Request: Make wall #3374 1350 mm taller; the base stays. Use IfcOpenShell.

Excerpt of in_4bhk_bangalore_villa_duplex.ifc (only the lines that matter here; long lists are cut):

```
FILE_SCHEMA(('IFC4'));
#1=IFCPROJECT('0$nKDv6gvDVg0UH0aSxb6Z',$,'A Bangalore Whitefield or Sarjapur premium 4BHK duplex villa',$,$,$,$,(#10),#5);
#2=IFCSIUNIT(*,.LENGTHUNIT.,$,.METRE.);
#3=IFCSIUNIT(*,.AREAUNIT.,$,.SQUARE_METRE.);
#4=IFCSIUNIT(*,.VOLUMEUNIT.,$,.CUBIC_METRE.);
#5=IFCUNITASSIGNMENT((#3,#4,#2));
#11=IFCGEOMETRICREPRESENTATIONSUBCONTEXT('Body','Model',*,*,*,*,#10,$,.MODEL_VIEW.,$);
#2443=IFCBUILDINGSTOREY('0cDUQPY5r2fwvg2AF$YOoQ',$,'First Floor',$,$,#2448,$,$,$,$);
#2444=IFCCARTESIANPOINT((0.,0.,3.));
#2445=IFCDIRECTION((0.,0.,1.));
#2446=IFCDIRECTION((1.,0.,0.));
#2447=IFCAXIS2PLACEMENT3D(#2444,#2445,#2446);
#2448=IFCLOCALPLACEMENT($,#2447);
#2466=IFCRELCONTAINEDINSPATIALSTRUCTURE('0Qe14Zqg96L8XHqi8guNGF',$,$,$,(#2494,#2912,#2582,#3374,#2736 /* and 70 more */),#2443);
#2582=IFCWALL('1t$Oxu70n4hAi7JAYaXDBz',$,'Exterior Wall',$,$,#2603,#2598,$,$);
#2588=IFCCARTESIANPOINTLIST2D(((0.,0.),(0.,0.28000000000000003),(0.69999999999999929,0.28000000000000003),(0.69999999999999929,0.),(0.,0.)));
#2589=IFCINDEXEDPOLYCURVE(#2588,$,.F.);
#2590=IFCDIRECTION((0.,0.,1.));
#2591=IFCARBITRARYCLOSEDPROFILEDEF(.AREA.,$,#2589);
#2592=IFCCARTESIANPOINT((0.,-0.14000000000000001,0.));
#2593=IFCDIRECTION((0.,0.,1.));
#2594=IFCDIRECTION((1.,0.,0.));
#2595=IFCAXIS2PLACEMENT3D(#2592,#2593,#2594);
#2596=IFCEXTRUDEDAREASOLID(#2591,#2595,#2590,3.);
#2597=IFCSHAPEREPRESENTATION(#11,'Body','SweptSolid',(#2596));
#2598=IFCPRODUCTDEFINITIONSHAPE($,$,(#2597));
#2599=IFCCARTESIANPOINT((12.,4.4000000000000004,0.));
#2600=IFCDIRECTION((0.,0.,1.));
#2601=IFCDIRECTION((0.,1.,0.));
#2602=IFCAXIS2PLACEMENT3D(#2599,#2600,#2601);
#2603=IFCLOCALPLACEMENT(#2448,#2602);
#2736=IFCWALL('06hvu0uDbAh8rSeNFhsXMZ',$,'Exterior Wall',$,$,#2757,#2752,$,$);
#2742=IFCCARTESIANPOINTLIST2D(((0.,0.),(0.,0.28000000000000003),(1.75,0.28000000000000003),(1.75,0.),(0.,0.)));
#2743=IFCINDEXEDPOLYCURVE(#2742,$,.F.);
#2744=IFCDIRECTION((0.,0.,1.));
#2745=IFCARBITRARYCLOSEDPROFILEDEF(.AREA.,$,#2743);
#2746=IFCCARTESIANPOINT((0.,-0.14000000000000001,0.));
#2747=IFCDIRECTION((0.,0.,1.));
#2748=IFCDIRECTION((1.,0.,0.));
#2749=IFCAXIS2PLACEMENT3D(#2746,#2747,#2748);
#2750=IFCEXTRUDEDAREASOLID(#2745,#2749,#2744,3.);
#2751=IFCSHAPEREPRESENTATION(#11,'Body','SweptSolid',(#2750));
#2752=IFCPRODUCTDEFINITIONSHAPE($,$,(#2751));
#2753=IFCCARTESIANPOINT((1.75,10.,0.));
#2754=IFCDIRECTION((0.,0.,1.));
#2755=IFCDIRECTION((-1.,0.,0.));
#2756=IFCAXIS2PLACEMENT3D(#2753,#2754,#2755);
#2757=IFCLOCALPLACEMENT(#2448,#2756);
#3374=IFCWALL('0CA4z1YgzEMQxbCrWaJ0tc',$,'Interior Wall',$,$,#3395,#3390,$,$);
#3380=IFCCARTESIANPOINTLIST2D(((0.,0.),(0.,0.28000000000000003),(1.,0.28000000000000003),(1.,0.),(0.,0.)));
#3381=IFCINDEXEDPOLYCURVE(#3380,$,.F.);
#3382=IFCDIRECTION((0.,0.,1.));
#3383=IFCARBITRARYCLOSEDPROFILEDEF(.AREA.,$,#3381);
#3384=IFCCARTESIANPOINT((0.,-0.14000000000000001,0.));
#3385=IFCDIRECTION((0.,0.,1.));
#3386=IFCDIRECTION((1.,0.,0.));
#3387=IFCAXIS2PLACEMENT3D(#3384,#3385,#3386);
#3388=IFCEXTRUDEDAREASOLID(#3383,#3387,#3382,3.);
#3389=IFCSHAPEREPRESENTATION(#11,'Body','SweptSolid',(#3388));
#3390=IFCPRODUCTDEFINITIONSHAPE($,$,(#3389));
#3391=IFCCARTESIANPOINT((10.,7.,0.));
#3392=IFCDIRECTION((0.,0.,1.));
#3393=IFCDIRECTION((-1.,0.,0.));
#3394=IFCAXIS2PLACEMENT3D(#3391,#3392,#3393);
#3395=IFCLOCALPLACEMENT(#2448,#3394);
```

```python
import ifcopenshell
import ifcopenshell.geom
import ifcopenshell.util.representation
import ifcopenshell.util.shape

model = ifcopenshell.open("in_4bhk_bangalore_villa_duplex.ifc")
settings = ifcopenshell.geom.settings()


def volume(element):
    """Net volume in cubic metres, openings subtracted."""
    shape = ifcopenshell.geom.create_shape(settings, element)
    return ifcopenshell.util.shape.get_volume(shape.geometry)


wall = model.by_guid("0CA4z1YgzEMQxbCrWaJ0tc")
before = volume(wall)

body = ifcopenshell.util.representation.get_representation(wall, "Model", "Body")
solid = body.Items[0]
old_height = solid.Depth
solid.Depth += 1.35
after = volume(wall)

print(f"height {old_height:g} -> {solid.Depth:g}, volume {before:.3f} -> {after:.3f} m3")

model.write("in_4bhk_bangalore_villa_duplex_rev.ifc")
```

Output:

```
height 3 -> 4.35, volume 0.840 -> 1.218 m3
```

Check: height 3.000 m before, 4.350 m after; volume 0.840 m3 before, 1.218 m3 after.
